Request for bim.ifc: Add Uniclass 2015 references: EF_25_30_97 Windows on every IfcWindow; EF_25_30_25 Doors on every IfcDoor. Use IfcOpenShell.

First a look at what the model holds.

```python
import ifcopenshell

model = ifcopenshell.open("bim.ifc")
print(model.schema)
print("classifications:", [c.Name for c in model.by_type("IfcClassification")])
for ifc_class in ("IfcDoor", "IfcRoof", "IfcStair", "IfcWall", "IfcWindow"):
    print(ifc_class, len(model.by_type(ifc_class)))
```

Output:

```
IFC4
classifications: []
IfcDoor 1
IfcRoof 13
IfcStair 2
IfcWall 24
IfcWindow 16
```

```python
import ifcopenshell
import ifcopenshell.api.classification

model = ifcopenshell.open("bim.ifc")

system = ifcopenshell.api.classification.add_classification(model, classification="Uniclass 2015")

codes = {
    "IfcWindow": ("EF_25_30_97", "Windows"),
    "IfcDoor": ("EF_25_30_25", "Doors"),
}
for ifc_class, (code, name) in codes.items():
    products = model.by_type(ifc_class)
    ifcopenshell.api.classification.add_reference(
        model, products=products, classification=system, identification=code, name=name
    )
    print(code, len(products))

model.write("bim-out.ifc")
```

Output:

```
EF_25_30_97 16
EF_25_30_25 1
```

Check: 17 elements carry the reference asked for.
